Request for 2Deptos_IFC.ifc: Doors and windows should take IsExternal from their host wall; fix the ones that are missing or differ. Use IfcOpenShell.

First a look at what the model holds.

```python
import ifcopenshell
import ifcopenshell.util.element

model = ifcopenshell.open("2Deptos_IFC.ifc")
print(model.schema)
seen = {}
for e in model.by_type("IfcDoor") + model.by_type("IfcWindow"):
    if not e.FillsVoids:
        continue
    host = e.FillsVoids[0].RelatingOpeningElement.VoidsElements[0].RelatingBuildingElement
    own = ifcopenshell.util.element.get_pset(e, f"Pset_{e.is_a()[3:].removesuffix('StandardCase')}Common", "IsExternal")
    wall = ifcopenshell.util.element.get_pset(host, "Pset_WallCommon", "IsExternal")
    seen[e.is_a(), own, wall] = seen.get((e.is_a(), own, wall), 0) + 1
for (cls, own, wall), count in sorted(seen.items(), key=str):
    print(count, cls, "IsExternal:", own, "| host wall:", wall)
```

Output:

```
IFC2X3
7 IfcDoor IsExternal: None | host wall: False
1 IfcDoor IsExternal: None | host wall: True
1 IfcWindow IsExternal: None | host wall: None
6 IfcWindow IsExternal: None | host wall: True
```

```python
import ifcopenshell
import ifcopenshell.api.pset
import ifcopenshell.util.element

model = ifcopenshell.open("2Deptos_IFC.ifc")

count = 0
for ifc_class, pset_name in (("IfcDoor", "Pset_DoorCommon"), ("IfcWindow", "Pset_WindowCommon")):
    for e in model.by_type(ifc_class):
        if not e.FillsVoids:
            continue
        host = e.FillsVoids[0].RelatingOpeningElement.VoidsElements[0].RelatingBuildingElement
        external = ifcopenshell.util.element.get_pset(host, "Pset_WallCommon", "IsExternal")
        if external is None or ifcopenshell.util.element.get_pset(e, pset_name, "IsExternal") == external:
            continue
        pset = ifcopenshell.api.pset.add_pset(model, product=e, name=pset_name)
        ifcopenshell.api.pset.edit_pset(model, pset=pset, properties={"IsExternal": external})
        count += 1

print(count, "updated")

model.write("2Deptos_IFC_v2.ifc")
```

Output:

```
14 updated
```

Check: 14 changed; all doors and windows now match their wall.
